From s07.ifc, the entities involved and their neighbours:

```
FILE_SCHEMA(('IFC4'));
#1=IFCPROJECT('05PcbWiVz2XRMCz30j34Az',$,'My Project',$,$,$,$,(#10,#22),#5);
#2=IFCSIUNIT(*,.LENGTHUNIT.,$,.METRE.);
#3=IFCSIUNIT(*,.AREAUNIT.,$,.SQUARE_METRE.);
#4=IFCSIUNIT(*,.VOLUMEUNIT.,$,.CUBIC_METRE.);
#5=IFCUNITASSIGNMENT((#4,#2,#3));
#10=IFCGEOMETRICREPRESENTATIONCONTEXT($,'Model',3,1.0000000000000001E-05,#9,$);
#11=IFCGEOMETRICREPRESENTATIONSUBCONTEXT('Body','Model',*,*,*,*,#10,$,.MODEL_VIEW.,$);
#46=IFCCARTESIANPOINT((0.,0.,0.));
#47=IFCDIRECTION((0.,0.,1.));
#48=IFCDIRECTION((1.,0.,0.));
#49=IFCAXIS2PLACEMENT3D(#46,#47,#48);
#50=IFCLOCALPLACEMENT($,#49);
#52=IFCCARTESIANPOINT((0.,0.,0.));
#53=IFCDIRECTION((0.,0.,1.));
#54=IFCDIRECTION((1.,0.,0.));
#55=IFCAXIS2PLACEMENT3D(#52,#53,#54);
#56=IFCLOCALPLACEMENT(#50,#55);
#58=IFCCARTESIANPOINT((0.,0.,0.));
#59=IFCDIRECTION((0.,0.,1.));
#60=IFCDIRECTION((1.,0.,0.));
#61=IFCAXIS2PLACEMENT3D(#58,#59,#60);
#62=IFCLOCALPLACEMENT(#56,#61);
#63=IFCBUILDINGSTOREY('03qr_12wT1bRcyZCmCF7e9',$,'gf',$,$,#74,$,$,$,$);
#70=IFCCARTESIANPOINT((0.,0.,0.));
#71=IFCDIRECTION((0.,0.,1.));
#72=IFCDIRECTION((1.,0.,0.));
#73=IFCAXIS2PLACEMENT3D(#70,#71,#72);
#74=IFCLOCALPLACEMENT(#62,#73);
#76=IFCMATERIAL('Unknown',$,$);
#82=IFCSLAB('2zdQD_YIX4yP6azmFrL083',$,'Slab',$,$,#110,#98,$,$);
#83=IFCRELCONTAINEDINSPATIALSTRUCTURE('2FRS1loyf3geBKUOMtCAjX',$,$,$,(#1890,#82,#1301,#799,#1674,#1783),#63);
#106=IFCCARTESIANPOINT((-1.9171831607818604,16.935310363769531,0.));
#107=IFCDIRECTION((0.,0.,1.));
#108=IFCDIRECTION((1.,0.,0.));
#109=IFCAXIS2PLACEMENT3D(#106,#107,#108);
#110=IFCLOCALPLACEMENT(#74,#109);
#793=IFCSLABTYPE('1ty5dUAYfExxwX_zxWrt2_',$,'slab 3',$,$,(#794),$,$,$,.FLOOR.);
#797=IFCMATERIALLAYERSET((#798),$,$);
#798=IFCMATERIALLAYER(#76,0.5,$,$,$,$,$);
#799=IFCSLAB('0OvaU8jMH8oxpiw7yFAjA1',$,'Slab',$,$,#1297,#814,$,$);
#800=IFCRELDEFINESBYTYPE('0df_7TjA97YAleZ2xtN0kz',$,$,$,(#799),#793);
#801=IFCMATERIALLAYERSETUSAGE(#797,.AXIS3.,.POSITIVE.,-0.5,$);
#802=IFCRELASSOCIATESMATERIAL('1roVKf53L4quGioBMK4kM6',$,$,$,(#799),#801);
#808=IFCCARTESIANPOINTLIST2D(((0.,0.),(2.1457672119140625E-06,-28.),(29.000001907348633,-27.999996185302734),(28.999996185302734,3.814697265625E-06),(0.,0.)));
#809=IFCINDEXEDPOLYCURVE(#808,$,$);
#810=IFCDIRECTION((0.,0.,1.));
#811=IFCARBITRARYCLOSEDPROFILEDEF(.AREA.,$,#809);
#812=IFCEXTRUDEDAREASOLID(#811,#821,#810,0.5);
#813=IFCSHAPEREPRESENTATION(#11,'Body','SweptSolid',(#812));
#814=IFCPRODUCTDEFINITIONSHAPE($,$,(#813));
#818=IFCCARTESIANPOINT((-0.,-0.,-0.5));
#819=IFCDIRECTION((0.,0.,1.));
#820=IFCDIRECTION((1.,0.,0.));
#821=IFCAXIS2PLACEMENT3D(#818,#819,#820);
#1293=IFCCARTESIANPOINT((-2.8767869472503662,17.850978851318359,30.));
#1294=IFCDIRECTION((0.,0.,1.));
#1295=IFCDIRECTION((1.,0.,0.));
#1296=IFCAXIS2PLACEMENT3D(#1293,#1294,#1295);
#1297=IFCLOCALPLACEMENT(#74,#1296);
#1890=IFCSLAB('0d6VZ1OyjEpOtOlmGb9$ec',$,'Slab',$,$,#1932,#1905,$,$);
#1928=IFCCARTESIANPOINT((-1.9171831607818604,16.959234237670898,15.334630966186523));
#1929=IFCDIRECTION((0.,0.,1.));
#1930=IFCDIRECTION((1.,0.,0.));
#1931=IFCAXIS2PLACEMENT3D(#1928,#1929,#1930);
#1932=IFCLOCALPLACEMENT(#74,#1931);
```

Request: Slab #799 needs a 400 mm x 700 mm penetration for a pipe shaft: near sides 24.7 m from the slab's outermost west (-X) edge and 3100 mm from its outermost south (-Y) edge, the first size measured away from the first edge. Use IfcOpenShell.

```python
import numpy as np
import ifcopenshell
import ifcopenshell.api.feature
import ifcopenshell.api.geometry
import ifcopenshell.api.root
import ifcopenshell.geom
import ifcopenshell.util.placement
import ifcopenshell.util.representation
import ifcopenshell.util.shape
import ifcopenshell.util.unit

model = ifcopenshell.open("s07.ifc")
unit_scale = ifcopenshell.util.unit.calculate_unit_scale(model)
settings = ifcopenshell.geom.settings()


def volume(element):
    """Net volume in cubic metres, openings subtracted."""
    shape = ifcopenshell.geom.create_shape(settings, element)
    return ifcopenshell.util.shape.get_volume(shape.geometry)


slab = model.by_guid("0OvaU8jMH8oxpiw7yFAjA1")
before = volume(slab)

# Extent in the slab's own axes, in metres. The edges named are its -X and -Y sides.
slab_shape = ifcopenshell.geom.create_shape(settings, slab)
vertices = ifcopenshell.util.shape.get_vertices(slab_shape.geometry)
x_min, y_min, bottom = vertices.min(axis=0)
top = vertices[:, 2].max()

opening = ifcopenshell.api.root.create_entity(model, ifc_class="IfcOpeningElement", name="Pipe shaft opening", predefined_type="OPENING")
context = ifcopenshell.util.representation.get_context(model, "Model", "Body", "MODEL_VIEW")
width, depth = 0.4, 0.7
outline = [(0.0, 0.0), (width, 0.0), (width, depth), (0.0, depth), (0.0, 0.0)]
# Overshoot both faces by 50 mm so the cut is clean.
shape = ifcopenshell.api.geometry.add_slab_representation(
    model, context=context, depth=top - bottom + 0.1, polyline=outline
)
ifcopenshell.api.geometry.assign_representation(model, product=opening, representation=shape)

matrix = ifcopenshell.util.placement.get_local_placement(slab.ObjectPlacement)
matrix[:, 3] = matrix @ np.append(np.array([x_min + 24.7, y_min + 3.1, bottom - 0.05]) / unit_scale, 1.0)
ifcopenshell.api.geometry.edit_object_placement(model, product=opening, matrix=matrix, is_si=False)
ifcopenshell.api.feature.add_feature(model, feature=opening, element=slab)

after = volume(slab)

print(f"slab volume {before:.3f} -> {after:.3f} m3")

model.write("s07_updated.ifc")
```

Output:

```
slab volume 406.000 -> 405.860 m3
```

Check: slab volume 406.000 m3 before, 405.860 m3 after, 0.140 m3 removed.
